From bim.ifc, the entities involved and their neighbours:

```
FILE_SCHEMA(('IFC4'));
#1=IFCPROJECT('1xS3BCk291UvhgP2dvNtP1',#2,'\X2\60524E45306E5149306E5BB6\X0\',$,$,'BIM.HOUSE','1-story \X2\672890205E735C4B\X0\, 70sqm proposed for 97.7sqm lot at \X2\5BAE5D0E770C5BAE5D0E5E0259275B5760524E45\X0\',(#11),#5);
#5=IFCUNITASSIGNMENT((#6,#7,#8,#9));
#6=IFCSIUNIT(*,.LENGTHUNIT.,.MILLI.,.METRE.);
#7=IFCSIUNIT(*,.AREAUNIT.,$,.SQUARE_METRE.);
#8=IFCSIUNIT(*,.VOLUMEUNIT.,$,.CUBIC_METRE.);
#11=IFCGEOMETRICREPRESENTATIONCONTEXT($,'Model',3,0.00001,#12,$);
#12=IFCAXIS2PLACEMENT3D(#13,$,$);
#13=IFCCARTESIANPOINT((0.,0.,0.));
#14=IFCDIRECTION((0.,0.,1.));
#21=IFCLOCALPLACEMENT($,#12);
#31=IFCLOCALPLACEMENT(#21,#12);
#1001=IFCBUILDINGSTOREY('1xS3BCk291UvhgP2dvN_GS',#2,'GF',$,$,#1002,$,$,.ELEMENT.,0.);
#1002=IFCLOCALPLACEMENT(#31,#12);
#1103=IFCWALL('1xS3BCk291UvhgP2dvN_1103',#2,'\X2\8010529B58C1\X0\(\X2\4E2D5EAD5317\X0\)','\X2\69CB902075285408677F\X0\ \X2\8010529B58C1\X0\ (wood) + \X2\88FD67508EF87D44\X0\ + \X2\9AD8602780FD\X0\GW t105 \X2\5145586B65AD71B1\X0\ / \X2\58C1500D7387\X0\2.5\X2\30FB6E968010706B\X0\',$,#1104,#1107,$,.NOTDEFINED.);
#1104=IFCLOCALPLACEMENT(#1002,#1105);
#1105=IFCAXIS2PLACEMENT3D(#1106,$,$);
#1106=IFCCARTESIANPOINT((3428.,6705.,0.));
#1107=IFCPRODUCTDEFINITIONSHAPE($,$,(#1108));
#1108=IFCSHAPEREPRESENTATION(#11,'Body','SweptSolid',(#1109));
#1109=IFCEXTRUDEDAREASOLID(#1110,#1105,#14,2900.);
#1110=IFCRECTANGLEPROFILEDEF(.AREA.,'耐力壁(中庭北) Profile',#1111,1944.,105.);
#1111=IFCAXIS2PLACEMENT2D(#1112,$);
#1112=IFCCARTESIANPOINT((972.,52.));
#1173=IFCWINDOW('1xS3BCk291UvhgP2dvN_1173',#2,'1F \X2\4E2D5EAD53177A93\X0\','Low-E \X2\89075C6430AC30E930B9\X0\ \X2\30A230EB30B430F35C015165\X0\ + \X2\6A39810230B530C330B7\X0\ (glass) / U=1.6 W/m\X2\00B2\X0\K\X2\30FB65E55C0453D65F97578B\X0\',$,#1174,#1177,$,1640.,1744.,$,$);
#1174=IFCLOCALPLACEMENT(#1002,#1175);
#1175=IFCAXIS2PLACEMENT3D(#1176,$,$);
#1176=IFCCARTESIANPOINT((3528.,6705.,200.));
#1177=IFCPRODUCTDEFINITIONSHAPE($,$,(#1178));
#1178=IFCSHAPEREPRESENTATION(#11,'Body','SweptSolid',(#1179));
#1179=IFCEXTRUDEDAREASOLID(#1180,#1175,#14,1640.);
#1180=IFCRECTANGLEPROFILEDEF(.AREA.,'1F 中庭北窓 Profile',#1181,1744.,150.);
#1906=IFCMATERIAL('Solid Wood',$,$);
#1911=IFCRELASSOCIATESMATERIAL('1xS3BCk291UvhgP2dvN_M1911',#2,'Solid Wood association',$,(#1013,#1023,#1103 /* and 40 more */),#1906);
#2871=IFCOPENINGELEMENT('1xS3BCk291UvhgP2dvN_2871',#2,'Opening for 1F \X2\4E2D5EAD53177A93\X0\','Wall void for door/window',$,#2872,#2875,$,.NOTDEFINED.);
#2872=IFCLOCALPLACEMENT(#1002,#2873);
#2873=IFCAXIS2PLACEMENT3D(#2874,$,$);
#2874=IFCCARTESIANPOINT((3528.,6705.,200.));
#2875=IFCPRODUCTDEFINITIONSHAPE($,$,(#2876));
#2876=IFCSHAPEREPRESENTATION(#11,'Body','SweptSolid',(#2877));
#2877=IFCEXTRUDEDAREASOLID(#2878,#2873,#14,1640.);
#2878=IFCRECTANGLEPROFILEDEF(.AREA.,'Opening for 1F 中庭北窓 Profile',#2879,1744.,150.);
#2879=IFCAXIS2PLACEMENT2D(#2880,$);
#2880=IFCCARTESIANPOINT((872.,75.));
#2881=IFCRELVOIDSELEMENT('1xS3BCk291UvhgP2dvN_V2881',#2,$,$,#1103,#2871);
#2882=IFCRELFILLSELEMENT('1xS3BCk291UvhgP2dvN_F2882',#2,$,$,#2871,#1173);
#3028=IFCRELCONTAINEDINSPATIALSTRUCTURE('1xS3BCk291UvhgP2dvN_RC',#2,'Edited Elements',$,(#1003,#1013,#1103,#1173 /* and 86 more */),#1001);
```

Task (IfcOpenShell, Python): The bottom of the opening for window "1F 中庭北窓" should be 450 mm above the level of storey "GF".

```python
import numpy as np
import ifcopenshell
import ifcopenshell.api.geometry
import ifcopenshell.geom
import ifcopenshell.util.element
import ifcopenshell.util.placement
import ifcopenshell.util.shape
import ifcopenshell.util.unit

model = ifcopenshell.open("bim.ifc")
unit_scale = ifcopenshell.util.unit.calculate_unit_scale(model)

window = model.by_guid("1xS3BCk291UvhgP2dvN_1173")
opening = window.FillsVoids[0].RelatingOpeningElement
storey = ifcopenshell.util.element.get_container(window, ifc_class="IfcBuildingStorey")
level = ifcopenshell.util.placement.get_local_placement(storey.ObjectPlacement)[2, 3]

# The opening's origin need not be at the sill, so measure its lowest point.
shape = ifcopenshell.geom.create_shape(ifcopenshell.geom.settings(), opening)
bottom = ifcopenshell.util.shape.get_shape_bottom_elevation(shape, shape.geometry) / unit_scale
dz = level + 0.45 / unit_scale - bottom

shift = np.array([0.0, 0.0, dz])
# The window is not placed relative to its opening, so move both.
for product in (opening, window):
    matrix = ifcopenshell.util.placement.get_local_placement(product.ObjectPlacement)
    matrix[:3, 3] += shift
    ifcopenshell.api.geometry.edit_object_placement(model, product=product, matrix=matrix, is_si=False)

print(f"moved by {dz * unit_scale:+.3f} m")

model.write("bim_rev.ifc")
```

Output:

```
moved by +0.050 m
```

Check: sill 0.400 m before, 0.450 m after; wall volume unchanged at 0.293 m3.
